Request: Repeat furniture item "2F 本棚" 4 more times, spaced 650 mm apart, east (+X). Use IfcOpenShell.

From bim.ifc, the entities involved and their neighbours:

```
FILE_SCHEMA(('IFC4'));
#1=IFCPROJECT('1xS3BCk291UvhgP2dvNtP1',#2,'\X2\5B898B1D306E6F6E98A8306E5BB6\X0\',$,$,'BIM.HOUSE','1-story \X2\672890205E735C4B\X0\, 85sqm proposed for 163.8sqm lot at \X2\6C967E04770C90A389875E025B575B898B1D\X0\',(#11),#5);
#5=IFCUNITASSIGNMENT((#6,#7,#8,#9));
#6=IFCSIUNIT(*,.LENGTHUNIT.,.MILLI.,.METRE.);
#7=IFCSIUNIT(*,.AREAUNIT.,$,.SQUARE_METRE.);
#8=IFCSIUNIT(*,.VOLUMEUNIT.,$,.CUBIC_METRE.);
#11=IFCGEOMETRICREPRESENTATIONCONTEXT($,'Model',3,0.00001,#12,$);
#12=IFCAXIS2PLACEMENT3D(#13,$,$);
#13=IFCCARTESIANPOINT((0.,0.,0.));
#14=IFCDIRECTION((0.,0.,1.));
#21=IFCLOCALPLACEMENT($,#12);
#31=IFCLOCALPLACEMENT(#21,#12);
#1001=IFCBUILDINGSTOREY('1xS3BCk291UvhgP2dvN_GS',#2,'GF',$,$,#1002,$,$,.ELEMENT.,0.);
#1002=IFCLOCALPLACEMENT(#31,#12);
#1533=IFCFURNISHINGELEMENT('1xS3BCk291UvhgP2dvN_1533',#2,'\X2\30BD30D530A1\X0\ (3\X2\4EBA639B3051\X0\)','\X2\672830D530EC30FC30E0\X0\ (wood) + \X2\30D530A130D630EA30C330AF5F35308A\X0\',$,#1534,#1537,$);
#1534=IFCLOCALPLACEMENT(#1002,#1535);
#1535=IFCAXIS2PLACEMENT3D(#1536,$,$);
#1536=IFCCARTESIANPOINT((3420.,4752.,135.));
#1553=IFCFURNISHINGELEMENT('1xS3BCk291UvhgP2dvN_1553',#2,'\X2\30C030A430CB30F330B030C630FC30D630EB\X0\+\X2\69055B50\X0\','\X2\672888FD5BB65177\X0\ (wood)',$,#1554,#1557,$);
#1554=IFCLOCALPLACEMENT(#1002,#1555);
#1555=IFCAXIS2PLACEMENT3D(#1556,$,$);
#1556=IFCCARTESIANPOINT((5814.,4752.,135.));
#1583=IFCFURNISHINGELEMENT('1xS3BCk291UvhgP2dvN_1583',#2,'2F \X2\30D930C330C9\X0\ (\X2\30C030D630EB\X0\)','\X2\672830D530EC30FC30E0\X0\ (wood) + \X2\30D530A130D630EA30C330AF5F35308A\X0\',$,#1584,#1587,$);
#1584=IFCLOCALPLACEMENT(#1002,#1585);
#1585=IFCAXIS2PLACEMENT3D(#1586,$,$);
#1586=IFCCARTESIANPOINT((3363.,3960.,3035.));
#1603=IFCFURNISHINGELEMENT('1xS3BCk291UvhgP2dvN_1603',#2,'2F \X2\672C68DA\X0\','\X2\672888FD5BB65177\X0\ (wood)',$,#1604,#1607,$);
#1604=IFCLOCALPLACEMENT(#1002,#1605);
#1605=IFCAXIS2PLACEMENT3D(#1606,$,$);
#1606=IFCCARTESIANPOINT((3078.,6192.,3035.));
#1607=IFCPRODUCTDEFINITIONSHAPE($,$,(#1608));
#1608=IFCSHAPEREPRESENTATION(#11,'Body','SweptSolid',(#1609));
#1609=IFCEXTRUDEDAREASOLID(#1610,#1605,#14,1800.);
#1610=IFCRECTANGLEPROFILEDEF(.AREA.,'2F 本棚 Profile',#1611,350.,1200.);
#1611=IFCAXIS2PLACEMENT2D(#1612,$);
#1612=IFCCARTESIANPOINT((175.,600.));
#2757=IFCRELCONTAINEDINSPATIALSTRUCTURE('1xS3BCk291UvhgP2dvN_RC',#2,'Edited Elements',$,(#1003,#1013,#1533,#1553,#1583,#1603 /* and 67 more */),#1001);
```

```python
import numpy as np
import ifcopenshell
import ifcopenshell.api.geometry
import ifcopenshell.api.root
import ifcopenshell.util.element
import ifcopenshell.util.placement
import ifcopenshell.util.unit

model = ifcopenshell.open("bim.ifc")
unit_scale = ifcopenshell.util.unit.calculate_unit_scale(model)


def reuse_history(source, copy):
    """copy_class also copies each property set's owner history, people and application; keep the originals."""
    for rel in copy.IsDefinedBy:
        if rel.is_a("IfcRelDefinesByProperties") and (history := rel.RelatingPropertyDefinition.OwnerHistory):
            rel.RelatingPropertyDefinition.OwnerHistory = source.OwnerHistory
            ifcopenshell.util.element.remove_deep2(model, history)


source = model.by_guid("1xS3BCk291UvhgP2dvN_1603")
base = ifcopenshell.util.placement.get_local_placement(source.ObjectPlacement)
step = np.array([1.0, 0.0, 0.0]) * 0.65 / unit_scale

for i in range(1, 5):
    copy = ifcopenshell.api.root.copy_class(model, product=source)
    copy.Representation = ifcopenshell.util.element.copy_deep(
        model, source.Representation, exclude=["IfcGeometricRepresentationContext", "IfcRepresentationMap"]
    )
    reuse_history(source, copy)
    matrix = base.copy()
    matrix[:3, 3] += i * step
    print("added at", matrix[:3, 3].round(3) + 0.0)
    ifcopenshell.api.geometry.edit_object_placement(model, product=copy, matrix=matrix, is_si=False)

model.write("bim_rev.ifc")
```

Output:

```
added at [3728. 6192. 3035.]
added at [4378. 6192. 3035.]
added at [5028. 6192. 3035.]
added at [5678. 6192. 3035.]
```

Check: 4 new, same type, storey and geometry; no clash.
